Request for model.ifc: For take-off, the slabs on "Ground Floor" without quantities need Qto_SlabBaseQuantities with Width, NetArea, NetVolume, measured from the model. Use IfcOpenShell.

First a look at what the model holds.

```python
import ifcopenshell
import ifcopenshell.util.element
import ifcopenshell.util.unit

model = ifcopenshell.open("model.ifc")
print(model.schema)
for unit_type in ("LENGTHUNIT", "AREAUNIT", "VOLUMEUNIT"):
    print(unit_type, ifcopenshell.util.unit.calculate_unit_scale(model, unit_type))
storey = next(s for s in model.by_type("IfcBuildingStorey") if s.Name == "Ground Floor")
slabs = [e for e in ifcopenshell.util.element.get_decomposition(storey) if e.is_a("IfcSlab")]
for e in sorted(slabs, key=lambda e: e.id()):
    print(e.id(), e.is_a(), e.Name, list(ifcopenshell.util.element.get_psets(e, qtos_only=True)), sep=" | ")
```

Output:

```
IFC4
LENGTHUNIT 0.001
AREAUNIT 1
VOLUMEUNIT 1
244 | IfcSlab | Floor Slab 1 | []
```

```python
import ifcopenshell
import ifcopenshell.api.pset
import ifcopenshell.geom
import ifcopenshell.util.element
import ifcopenshell.util.shape
import ifcopenshell.util.unit

model = ifcopenshell.open("model.ifc")
unit_scale = ifcopenshell.util.unit.calculate_unit_scale(model)
area_scale = ifcopenshell.util.unit.calculate_unit_scale(model, "AREAUNIT")
volume_scale = ifcopenshell.util.unit.calculate_unit_scale(model, "VOLUMEUNIT")
settings = ifcopenshell.geom.settings()

storey = next(s for s in model.by_type("IfcBuildingStorey") if s.Name == "Ground Floor")
slabs = [e for e in ifcopenshell.util.element.get_decomposition(storey) if e.is_a("IfcSlab")]

for e in sorted(slabs, key=lambda e: e.id()):
    if ifcopenshell.util.element.get_psets(e, qtos_only=True, should_inherit=False):
        continue
    # Geometry comes back in metres, in the element's own axes.
    shape = ifcopenshell.geom.create_shape(settings, e)
    values = {
        "Width": ifcopenshell.util.shape.get_z(shape.geometry) / unit_scale,
        "NetArea": ifcopenshell.util.shape.get_footprint_area(shape.geometry) / area_scale,
        "NetVolume": ifcopenshell.util.shape.get_volume(shape.geometry) / volume_scale,
    }
    qto = ifcopenshell.api.pset.add_qto(model, product=e, name="Qto_SlabBaseQuantities")
    ifcopenshell.api.pset.edit_qto(model, qto=qto, properties=values)
    print(e.id(), {k: round(v, 3) for k, v in values.items()})

model.write("model_rev.ifc")
```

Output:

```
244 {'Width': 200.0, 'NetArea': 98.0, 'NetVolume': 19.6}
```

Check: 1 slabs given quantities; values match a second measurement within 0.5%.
